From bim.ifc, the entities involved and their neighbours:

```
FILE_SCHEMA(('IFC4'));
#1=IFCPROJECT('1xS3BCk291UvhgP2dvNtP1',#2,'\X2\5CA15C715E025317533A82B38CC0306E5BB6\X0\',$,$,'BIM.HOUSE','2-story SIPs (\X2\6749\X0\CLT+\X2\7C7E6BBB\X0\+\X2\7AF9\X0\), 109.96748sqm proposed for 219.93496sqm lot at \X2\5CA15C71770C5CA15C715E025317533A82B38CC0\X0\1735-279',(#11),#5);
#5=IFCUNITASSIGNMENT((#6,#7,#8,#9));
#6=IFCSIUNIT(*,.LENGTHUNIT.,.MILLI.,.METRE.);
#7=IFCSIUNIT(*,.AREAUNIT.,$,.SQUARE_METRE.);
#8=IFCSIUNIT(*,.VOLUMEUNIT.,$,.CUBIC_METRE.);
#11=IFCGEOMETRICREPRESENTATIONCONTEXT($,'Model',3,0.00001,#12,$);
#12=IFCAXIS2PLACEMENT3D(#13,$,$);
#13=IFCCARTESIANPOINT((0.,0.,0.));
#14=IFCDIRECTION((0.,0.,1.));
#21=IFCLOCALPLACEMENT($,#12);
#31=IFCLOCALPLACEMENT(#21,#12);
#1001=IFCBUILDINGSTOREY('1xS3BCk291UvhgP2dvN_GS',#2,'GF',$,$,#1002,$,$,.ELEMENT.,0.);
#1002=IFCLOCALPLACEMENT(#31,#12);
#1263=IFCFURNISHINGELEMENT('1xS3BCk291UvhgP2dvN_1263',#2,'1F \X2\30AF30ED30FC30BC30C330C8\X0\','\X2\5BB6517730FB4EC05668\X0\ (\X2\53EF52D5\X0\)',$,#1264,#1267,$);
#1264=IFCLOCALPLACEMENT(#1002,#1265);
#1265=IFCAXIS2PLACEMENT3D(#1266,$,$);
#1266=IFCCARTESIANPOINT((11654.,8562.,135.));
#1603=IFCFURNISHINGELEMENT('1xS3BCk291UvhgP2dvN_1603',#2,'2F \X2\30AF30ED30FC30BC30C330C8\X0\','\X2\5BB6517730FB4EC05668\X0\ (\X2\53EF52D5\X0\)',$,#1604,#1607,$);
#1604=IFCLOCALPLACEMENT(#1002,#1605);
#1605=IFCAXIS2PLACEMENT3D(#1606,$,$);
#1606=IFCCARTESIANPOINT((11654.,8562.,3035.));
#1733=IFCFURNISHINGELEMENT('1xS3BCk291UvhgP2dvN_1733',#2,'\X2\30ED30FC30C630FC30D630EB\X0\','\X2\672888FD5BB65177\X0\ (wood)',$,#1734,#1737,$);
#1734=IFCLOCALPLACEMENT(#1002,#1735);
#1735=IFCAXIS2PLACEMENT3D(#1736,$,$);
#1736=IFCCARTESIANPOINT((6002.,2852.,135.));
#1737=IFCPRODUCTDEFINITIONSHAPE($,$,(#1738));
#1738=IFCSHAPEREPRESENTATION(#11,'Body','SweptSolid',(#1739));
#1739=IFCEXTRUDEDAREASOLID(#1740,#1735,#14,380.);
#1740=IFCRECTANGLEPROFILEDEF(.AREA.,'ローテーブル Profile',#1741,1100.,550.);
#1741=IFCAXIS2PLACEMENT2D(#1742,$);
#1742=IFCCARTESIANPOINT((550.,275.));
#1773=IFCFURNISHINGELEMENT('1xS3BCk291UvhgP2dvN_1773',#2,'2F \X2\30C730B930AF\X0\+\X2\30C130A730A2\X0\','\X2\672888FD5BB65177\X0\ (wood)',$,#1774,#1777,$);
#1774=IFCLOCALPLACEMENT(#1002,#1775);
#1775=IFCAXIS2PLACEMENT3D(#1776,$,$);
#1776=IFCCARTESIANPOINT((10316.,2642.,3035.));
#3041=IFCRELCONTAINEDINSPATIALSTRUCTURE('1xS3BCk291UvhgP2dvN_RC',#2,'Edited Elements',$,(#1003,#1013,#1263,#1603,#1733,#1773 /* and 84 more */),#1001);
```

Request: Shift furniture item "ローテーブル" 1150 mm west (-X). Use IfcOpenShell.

```python
import ifcopenshell
import ifcopenshell.api.geometry
import ifcopenshell.util.placement

model = ifcopenshell.open("bim.ifc")

item = model.by_id(1733)
matrix = ifcopenshell.util.placement.get_local_placement(item.ObjectPlacement)
matrix[0, 3] -= 1150.0
ifcopenshell.api.geometry.edit_object_placement(model, product=item, matrix=matrix, is_si=False)

print(ifcopenshell.util.placement.get_local_placement(item.ObjectPlacement).round(3) + 0.0)

model.write("bim_rev.ifc")
```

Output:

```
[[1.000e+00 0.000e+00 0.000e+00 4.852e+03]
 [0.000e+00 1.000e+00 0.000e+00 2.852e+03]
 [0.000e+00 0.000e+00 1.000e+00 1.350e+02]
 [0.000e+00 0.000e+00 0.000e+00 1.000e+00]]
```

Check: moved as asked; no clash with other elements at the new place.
